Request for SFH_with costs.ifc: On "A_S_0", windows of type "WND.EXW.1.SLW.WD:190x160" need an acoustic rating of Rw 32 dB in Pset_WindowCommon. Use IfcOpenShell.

First a look at what the model holds.

```python
import ifcopenshell
import ifcopenshell.util.element

model = ifcopenshell.open("SFH_with costs.ifc")
print(model.schema)
storey = next(s for s in model.by_type("IfcBuildingStorey") if s.Name == "A_S_0")
windows = [e for e in ifcopenshell.util.element.get_decomposition(storey) if e.is_a("IfcWindow")]
seen = {}
for e in windows:
    element_type = ifcopenshell.util.element.get_type(e)
    key = (element_type.Name if element_type != e and element_type else None, ifcopenshell.util.element.get_pset(e, "Pset_WindowCommon", "AcousticRating"))
    seen[key] = seen.get(key, 0) + 1
for (name, value), count in sorted(seen.items(), key=str):
    print(count, "x", name, "|", value)
```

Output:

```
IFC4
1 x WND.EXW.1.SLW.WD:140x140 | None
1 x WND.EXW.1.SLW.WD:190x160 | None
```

```python
import ifcopenshell
import ifcopenshell.api.pset
import ifcopenshell.util.element

model = ifcopenshell.open("SFH_with costs.ifc")

storey = next(s for s in model.by_type("IfcBuildingStorey") if s.Name == "A_S_0")
windows = [e for e in ifcopenshell.util.element.get_decomposition(storey) if e.is_a("IfcWindow")]

count = 0
for e in windows:
    element_type = ifcopenshell.util.element.get_type(e)
    if element_type in (None, e) or element_type.Name != "WND.EXW.1.SLW.WD:190x160":
        continue
    # add_pset returns the element's existing set when there is one.
    pset = ifcopenshell.api.pset.add_pset(model, product=e, name="Pset_WindowCommon")
    ifcopenshell.api.pset.edit_pset(model, pset=pset, properties={"AcousticRating": "Rw 32 dB"})
    count += 1

print(count, "windows updated")

model.write("SFH_with costs_edited.ifc")
```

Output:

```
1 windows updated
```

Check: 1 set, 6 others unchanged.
